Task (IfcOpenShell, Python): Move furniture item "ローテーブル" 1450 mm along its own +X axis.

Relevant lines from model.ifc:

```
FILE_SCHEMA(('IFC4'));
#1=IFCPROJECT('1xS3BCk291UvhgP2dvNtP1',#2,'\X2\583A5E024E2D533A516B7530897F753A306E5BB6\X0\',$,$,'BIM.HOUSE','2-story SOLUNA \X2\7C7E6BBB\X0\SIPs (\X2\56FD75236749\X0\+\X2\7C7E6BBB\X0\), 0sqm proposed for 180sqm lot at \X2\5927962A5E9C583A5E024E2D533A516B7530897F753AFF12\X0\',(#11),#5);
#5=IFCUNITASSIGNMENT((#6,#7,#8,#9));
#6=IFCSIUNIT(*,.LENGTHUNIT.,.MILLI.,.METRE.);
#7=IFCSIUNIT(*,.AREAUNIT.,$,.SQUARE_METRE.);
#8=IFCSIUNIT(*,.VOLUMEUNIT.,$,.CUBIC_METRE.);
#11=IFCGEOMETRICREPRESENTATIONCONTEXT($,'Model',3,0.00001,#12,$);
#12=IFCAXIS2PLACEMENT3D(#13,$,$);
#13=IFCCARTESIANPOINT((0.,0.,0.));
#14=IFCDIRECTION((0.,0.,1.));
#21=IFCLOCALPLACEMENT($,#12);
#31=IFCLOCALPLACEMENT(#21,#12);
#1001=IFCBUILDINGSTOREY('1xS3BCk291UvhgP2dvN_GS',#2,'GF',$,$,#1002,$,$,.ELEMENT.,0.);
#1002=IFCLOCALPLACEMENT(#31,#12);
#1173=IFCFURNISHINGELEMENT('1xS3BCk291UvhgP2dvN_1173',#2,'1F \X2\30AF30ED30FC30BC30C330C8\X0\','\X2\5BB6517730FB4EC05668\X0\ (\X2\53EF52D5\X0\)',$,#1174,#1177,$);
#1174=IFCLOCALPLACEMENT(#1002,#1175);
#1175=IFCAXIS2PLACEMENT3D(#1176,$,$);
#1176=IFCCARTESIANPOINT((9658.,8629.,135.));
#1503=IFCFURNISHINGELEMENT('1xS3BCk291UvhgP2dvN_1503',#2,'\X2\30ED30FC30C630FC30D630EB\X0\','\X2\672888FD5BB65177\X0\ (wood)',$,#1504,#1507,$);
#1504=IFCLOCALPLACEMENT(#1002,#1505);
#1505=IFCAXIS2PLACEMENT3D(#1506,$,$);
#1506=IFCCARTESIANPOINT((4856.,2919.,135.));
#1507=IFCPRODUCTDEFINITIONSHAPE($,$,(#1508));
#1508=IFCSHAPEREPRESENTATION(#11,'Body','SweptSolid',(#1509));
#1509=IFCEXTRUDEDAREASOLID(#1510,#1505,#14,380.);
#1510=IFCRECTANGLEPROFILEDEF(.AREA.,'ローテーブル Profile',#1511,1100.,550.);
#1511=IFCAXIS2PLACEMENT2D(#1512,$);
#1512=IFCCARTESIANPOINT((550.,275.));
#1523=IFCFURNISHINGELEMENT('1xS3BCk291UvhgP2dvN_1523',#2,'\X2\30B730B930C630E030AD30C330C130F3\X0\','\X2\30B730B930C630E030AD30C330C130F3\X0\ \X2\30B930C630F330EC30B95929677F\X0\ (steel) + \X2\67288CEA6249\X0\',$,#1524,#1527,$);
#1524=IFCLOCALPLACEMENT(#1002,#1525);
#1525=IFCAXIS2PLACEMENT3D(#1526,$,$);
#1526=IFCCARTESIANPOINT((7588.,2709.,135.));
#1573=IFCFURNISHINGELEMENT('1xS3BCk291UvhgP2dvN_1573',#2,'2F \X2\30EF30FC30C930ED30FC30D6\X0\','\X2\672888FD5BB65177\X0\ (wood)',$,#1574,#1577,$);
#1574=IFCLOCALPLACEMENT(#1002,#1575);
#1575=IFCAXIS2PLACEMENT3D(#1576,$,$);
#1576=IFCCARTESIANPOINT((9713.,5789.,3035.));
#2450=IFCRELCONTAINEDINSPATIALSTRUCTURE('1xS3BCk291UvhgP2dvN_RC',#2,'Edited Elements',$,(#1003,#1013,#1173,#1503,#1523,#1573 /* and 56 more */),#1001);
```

```python
import ifcopenshell
import ifcopenshell.api.geometry
import ifcopenshell.util.placement

model = ifcopenshell.open("model.ifc")

item = model.by_id(1503)
matrix = ifcopenshell.util.placement.get_local_placement(item.ObjectPlacement)
matrix[:3, 3] += matrix[:3, 0] * 1450.0
ifcopenshell.api.geometry.edit_object_placement(model, product=item, matrix=matrix, is_si=False)

print(ifcopenshell.util.placement.get_local_placement(item.ObjectPlacement).round(3) + 0.0)

model.write("model-out.ifc")
```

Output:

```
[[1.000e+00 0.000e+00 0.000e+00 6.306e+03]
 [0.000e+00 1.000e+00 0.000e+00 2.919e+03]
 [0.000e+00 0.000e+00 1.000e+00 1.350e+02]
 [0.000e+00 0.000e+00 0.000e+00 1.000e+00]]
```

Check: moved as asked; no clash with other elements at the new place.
